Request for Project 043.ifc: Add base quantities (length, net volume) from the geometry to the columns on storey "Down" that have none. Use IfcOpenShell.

First a look at what the model holds.

```python
import ifcopenshell
import ifcopenshell.util.element
import ifcopenshell.util.unit

model = ifcopenshell.open("Project 043.ifc")
print(model.schema)
for unit_type in ("LENGTHUNIT", "AREAUNIT", "VOLUMEUNIT"):
    print(unit_type, ifcopenshell.util.unit.calculate_unit_scale(model, unit_type))
storey = next(s for s in model.by_type("IfcBuildingStorey") if s.Name == "Down")
columns = [e for e in ifcopenshell.util.element.get_decomposition(storey) if e.is_a("IfcColumn")]
for e in sorted(columns, key=lambda e: e.id()):
    print(e.id(), e.is_a(), e.Name, list(ifcopenshell.util.element.get_psets(e, qtos_only=True)), sep=" | ")
```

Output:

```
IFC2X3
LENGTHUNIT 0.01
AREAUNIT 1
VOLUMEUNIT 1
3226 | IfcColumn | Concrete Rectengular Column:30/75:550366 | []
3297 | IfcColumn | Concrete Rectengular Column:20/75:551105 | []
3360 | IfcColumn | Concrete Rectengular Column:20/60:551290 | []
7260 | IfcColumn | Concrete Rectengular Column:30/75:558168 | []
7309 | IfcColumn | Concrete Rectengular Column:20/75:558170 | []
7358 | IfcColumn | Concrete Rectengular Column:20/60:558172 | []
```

```python
import ifcopenshell
import ifcopenshell.api.pset
import ifcopenshell.geom
import ifcopenshell.util.element
import ifcopenshell.util.shape
import ifcopenshell.util.unit

model = ifcopenshell.open("Project 043.ifc")
unit_scale = ifcopenshell.util.unit.calculate_unit_scale(model)
volume_scale = ifcopenshell.util.unit.calculate_unit_scale(model, "VOLUMEUNIT")
settings = ifcopenshell.geom.settings()

storey = next(s for s in model.by_type("IfcBuildingStorey") if s.Name == "Down")
columns = [e for e in ifcopenshell.util.element.get_decomposition(storey) if e.is_a("IfcColumn")]

for e in sorted(columns, key=lambda e: e.id()):
    if ifcopenshell.util.element.get_psets(e, qtos_only=True, should_inherit=False):
        continue
    # Geometry comes back in metres, in the element's own axes.
    shape = ifcopenshell.geom.create_shape(settings, e)
    values = {
        "Length": ifcopenshell.util.shape.get_z(shape.geometry) / unit_scale,
        "NetVolume": ifcopenshell.util.shape.get_volume(shape.geometry) / volume_scale,
    }
    qto = ifcopenshell.api.pset.add_qto(model, product=e, name="BaseQuantities")
    ifcopenshell.api.pset.edit_qto(model, qto=qto, properties=values)
    print(e.id(), {k: round(v, 3) for k, v in values.items()})

model.write("Project 043_rev.ifc")
```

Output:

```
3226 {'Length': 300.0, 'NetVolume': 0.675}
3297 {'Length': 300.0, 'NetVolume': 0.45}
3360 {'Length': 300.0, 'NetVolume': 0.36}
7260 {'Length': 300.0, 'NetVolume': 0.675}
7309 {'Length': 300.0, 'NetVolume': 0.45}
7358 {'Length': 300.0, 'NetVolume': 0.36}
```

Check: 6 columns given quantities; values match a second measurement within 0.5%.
